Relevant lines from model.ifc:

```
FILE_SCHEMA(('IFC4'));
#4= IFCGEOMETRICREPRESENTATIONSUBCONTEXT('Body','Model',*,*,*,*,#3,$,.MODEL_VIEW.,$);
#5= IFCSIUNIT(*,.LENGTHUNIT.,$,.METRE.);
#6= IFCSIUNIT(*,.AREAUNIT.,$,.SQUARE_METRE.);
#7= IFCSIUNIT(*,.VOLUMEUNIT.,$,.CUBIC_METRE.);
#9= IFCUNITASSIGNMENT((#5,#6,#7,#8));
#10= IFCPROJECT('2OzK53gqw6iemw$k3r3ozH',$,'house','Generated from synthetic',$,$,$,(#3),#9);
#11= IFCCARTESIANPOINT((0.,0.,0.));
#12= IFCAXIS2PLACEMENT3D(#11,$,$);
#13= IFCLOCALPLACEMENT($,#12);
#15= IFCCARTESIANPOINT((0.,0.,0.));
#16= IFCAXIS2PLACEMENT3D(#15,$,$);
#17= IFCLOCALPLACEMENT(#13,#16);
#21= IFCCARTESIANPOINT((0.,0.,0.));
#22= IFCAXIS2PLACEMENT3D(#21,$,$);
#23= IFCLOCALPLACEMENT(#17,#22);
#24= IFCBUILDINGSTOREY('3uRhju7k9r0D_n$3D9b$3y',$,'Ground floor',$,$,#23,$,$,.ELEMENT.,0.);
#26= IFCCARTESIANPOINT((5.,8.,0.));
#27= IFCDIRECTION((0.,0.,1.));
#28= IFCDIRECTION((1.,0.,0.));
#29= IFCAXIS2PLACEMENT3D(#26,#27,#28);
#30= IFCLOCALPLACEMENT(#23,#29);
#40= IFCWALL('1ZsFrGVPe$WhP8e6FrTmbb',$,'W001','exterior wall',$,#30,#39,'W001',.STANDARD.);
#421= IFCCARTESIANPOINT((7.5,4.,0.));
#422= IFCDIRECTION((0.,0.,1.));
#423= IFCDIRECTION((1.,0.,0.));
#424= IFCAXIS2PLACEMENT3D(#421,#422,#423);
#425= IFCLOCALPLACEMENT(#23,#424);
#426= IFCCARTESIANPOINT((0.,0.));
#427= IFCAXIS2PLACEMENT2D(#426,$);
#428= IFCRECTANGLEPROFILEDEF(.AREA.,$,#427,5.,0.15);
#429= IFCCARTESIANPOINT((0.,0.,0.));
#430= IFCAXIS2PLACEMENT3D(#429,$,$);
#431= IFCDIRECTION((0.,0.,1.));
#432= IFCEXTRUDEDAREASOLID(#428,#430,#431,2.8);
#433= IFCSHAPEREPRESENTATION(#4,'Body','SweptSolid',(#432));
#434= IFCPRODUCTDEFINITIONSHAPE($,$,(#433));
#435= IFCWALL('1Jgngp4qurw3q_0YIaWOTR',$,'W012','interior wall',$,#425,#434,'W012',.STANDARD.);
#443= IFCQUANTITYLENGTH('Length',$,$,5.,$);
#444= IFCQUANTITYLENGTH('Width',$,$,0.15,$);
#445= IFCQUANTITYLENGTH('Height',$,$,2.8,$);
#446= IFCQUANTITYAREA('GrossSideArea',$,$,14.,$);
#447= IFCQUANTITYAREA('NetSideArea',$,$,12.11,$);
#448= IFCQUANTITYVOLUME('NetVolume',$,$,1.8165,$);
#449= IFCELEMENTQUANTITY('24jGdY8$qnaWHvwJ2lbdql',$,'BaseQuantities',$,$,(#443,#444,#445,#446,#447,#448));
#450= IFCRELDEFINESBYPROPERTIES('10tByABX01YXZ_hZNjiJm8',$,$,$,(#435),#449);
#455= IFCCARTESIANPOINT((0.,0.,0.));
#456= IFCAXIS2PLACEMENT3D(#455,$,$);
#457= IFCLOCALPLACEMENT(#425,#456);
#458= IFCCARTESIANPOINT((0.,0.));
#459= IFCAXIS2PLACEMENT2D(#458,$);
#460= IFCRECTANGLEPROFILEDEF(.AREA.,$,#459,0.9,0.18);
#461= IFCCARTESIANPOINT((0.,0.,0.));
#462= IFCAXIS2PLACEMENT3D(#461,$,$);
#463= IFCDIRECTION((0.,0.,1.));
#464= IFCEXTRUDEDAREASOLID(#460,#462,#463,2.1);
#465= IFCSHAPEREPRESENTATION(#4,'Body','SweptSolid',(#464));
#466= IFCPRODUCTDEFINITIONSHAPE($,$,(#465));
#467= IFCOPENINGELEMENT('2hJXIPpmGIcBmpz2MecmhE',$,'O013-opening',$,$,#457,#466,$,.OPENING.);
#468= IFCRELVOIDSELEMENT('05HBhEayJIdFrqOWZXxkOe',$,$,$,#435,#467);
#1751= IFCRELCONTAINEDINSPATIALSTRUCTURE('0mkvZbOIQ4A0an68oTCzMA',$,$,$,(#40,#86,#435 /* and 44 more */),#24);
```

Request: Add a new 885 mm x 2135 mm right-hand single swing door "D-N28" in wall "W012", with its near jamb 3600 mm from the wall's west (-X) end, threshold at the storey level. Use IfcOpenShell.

```python
import numpy as np
import ifcopenshell
import ifcopenshell.api.feature
import ifcopenshell.api.geometry
import ifcopenshell.api.pset
import ifcopenshell.api.root
import ifcopenshell.api.spatial
import ifcopenshell.geom
import ifcopenshell.util.element
import ifcopenshell.util.placement
import ifcopenshell.util.representation
import ifcopenshell.util.shape
import ifcopenshell.util.unit

model = ifcopenshell.open("model.ifc")
unit_scale = ifcopenshell.util.unit.calculate_unit_scale(model)
area_scale = ifcopenshell.util.unit.calculate_unit_scale(model, "AREAUNIT")
volume_scale = ifcopenshell.util.unit.calculate_unit_scale(model, "VOLUMEUNIT")
settings = ifcopenshell.geom.settings()


def volume(element):
    """Net volume in cubic metres, openings subtracted."""
    shape = ifcopenshell.geom.create_shape(settings, element)
    return ifcopenshell.util.shape.get_volume(shape.geometry)


wall = model.by_guid("1Jgngp4qurw3q_0YIaWOTR")
storey = ifcopenshell.util.element.get_container(wall, ifc_class="IfcBuildingStorey")
context = ifcopenshell.util.representation.get_context(model, "Model", "Body", "MODEL_VIEW")
before = volume(wall)

width, height, from_end, sill = 0.885, 2.135, 3.6, 0.0  # metres

# The wall runs along its own X axis, and the end named is its -X end.
wall_shape = ifcopenshell.geom.create_shape(settings, wall)
x, y, z = ifcopenshell.util.shape.get_vertices(wall_shape.geometry).T
start = x.min() + from_end
face, thickness = float(y.min()), float(y.max() - y.min())
wall_matrix = ifcopenshell.util.placement.get_local_placement(wall.ObjectPlacement)
level = ifcopenshell.util.placement.get_local_placement(storey.ObjectPlacement)[2, 3]


def in_wall(x, y):
    """Placement at x, y metres in the wall's axes, at sill height."""
    matrix = wall_matrix.copy()
    matrix[:, 3] = wall_matrix @ np.array([x / unit_scale, y / unit_scale, 0.0, 1.0])
    matrix[2, 3] = level + sill / unit_scale
    return matrix


# Opening: a box that overshoots both wall faces by 50 mm.
opening = ifcopenshell.api.root.create_entity(model, ifc_class="IfcOpeningElement", predefined_type="OPENING")
box = ifcopenshell.api.geometry.add_wall_representation(
    model, context=context, length=width, height=height, thickness=thickness + 0.1
)
ifcopenshell.api.geometry.assign_representation(model, product=opening, representation=box)
ifcopenshell.api.geometry.edit_object_placement(model, product=opening, matrix=in_wall(start, face - 0.05), is_si=False)
ifcopenshell.api.feature.add_feature(model, feature=opening, element=wall)

door = ifcopenshell.api.root.create_entity(model, ifc_class="IfcDoor", name="D-N28", predefined_type="DOOR")
door.OverallWidth, door.OverallHeight = width / unit_scale, height / unit_scale
door.OperationType = "SINGLE_SWING_RIGHT"
body = ifcopenshell.api.geometry.add_door_representation(
    model,
    context=context,
    overall_width=door.OverallWidth,
    overall_height=door.OverallHeight,
    operation_type="SINGLE_SWING_RIGHT",
    lining_properties={"LiningDepth": thickness / unit_scale, "ThresholdDepth": thickness / unit_scale},
)
ifcopenshell.api.geometry.assign_representation(model, product=door, representation=body)
ifcopenshell.api.spatial.assign_container(model, products=[door], relating_structure=storey)
ifcopenshell.api.feature.add_filling(model, opening=opening, element=door)

# The lining spans the wall, so the door starts at the wall face.
ifcopenshell.api.geometry.edit_object_placement(model, product=door, matrix=in_wall(start, face), is_si=False)

after = volume(wall)

# Update the wall's stored quantities.
qto = model.by_id(ifcopenshell.util.element.get_pset(wall, "BaseQuantities", should_inherit=False)["id"])
ifcopenshell.api.pset.edit_qto(model, qto=qto, properties={
    "NetSideArea": after / thickness / area_scale,
    "NetVolume": after / volume_scale,
})

print(f"wall volume {before:.3f} -> {after:.3f} m3")

model.write("model_updated.ifc")
```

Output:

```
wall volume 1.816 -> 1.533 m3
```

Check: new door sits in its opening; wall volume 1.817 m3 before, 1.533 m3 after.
